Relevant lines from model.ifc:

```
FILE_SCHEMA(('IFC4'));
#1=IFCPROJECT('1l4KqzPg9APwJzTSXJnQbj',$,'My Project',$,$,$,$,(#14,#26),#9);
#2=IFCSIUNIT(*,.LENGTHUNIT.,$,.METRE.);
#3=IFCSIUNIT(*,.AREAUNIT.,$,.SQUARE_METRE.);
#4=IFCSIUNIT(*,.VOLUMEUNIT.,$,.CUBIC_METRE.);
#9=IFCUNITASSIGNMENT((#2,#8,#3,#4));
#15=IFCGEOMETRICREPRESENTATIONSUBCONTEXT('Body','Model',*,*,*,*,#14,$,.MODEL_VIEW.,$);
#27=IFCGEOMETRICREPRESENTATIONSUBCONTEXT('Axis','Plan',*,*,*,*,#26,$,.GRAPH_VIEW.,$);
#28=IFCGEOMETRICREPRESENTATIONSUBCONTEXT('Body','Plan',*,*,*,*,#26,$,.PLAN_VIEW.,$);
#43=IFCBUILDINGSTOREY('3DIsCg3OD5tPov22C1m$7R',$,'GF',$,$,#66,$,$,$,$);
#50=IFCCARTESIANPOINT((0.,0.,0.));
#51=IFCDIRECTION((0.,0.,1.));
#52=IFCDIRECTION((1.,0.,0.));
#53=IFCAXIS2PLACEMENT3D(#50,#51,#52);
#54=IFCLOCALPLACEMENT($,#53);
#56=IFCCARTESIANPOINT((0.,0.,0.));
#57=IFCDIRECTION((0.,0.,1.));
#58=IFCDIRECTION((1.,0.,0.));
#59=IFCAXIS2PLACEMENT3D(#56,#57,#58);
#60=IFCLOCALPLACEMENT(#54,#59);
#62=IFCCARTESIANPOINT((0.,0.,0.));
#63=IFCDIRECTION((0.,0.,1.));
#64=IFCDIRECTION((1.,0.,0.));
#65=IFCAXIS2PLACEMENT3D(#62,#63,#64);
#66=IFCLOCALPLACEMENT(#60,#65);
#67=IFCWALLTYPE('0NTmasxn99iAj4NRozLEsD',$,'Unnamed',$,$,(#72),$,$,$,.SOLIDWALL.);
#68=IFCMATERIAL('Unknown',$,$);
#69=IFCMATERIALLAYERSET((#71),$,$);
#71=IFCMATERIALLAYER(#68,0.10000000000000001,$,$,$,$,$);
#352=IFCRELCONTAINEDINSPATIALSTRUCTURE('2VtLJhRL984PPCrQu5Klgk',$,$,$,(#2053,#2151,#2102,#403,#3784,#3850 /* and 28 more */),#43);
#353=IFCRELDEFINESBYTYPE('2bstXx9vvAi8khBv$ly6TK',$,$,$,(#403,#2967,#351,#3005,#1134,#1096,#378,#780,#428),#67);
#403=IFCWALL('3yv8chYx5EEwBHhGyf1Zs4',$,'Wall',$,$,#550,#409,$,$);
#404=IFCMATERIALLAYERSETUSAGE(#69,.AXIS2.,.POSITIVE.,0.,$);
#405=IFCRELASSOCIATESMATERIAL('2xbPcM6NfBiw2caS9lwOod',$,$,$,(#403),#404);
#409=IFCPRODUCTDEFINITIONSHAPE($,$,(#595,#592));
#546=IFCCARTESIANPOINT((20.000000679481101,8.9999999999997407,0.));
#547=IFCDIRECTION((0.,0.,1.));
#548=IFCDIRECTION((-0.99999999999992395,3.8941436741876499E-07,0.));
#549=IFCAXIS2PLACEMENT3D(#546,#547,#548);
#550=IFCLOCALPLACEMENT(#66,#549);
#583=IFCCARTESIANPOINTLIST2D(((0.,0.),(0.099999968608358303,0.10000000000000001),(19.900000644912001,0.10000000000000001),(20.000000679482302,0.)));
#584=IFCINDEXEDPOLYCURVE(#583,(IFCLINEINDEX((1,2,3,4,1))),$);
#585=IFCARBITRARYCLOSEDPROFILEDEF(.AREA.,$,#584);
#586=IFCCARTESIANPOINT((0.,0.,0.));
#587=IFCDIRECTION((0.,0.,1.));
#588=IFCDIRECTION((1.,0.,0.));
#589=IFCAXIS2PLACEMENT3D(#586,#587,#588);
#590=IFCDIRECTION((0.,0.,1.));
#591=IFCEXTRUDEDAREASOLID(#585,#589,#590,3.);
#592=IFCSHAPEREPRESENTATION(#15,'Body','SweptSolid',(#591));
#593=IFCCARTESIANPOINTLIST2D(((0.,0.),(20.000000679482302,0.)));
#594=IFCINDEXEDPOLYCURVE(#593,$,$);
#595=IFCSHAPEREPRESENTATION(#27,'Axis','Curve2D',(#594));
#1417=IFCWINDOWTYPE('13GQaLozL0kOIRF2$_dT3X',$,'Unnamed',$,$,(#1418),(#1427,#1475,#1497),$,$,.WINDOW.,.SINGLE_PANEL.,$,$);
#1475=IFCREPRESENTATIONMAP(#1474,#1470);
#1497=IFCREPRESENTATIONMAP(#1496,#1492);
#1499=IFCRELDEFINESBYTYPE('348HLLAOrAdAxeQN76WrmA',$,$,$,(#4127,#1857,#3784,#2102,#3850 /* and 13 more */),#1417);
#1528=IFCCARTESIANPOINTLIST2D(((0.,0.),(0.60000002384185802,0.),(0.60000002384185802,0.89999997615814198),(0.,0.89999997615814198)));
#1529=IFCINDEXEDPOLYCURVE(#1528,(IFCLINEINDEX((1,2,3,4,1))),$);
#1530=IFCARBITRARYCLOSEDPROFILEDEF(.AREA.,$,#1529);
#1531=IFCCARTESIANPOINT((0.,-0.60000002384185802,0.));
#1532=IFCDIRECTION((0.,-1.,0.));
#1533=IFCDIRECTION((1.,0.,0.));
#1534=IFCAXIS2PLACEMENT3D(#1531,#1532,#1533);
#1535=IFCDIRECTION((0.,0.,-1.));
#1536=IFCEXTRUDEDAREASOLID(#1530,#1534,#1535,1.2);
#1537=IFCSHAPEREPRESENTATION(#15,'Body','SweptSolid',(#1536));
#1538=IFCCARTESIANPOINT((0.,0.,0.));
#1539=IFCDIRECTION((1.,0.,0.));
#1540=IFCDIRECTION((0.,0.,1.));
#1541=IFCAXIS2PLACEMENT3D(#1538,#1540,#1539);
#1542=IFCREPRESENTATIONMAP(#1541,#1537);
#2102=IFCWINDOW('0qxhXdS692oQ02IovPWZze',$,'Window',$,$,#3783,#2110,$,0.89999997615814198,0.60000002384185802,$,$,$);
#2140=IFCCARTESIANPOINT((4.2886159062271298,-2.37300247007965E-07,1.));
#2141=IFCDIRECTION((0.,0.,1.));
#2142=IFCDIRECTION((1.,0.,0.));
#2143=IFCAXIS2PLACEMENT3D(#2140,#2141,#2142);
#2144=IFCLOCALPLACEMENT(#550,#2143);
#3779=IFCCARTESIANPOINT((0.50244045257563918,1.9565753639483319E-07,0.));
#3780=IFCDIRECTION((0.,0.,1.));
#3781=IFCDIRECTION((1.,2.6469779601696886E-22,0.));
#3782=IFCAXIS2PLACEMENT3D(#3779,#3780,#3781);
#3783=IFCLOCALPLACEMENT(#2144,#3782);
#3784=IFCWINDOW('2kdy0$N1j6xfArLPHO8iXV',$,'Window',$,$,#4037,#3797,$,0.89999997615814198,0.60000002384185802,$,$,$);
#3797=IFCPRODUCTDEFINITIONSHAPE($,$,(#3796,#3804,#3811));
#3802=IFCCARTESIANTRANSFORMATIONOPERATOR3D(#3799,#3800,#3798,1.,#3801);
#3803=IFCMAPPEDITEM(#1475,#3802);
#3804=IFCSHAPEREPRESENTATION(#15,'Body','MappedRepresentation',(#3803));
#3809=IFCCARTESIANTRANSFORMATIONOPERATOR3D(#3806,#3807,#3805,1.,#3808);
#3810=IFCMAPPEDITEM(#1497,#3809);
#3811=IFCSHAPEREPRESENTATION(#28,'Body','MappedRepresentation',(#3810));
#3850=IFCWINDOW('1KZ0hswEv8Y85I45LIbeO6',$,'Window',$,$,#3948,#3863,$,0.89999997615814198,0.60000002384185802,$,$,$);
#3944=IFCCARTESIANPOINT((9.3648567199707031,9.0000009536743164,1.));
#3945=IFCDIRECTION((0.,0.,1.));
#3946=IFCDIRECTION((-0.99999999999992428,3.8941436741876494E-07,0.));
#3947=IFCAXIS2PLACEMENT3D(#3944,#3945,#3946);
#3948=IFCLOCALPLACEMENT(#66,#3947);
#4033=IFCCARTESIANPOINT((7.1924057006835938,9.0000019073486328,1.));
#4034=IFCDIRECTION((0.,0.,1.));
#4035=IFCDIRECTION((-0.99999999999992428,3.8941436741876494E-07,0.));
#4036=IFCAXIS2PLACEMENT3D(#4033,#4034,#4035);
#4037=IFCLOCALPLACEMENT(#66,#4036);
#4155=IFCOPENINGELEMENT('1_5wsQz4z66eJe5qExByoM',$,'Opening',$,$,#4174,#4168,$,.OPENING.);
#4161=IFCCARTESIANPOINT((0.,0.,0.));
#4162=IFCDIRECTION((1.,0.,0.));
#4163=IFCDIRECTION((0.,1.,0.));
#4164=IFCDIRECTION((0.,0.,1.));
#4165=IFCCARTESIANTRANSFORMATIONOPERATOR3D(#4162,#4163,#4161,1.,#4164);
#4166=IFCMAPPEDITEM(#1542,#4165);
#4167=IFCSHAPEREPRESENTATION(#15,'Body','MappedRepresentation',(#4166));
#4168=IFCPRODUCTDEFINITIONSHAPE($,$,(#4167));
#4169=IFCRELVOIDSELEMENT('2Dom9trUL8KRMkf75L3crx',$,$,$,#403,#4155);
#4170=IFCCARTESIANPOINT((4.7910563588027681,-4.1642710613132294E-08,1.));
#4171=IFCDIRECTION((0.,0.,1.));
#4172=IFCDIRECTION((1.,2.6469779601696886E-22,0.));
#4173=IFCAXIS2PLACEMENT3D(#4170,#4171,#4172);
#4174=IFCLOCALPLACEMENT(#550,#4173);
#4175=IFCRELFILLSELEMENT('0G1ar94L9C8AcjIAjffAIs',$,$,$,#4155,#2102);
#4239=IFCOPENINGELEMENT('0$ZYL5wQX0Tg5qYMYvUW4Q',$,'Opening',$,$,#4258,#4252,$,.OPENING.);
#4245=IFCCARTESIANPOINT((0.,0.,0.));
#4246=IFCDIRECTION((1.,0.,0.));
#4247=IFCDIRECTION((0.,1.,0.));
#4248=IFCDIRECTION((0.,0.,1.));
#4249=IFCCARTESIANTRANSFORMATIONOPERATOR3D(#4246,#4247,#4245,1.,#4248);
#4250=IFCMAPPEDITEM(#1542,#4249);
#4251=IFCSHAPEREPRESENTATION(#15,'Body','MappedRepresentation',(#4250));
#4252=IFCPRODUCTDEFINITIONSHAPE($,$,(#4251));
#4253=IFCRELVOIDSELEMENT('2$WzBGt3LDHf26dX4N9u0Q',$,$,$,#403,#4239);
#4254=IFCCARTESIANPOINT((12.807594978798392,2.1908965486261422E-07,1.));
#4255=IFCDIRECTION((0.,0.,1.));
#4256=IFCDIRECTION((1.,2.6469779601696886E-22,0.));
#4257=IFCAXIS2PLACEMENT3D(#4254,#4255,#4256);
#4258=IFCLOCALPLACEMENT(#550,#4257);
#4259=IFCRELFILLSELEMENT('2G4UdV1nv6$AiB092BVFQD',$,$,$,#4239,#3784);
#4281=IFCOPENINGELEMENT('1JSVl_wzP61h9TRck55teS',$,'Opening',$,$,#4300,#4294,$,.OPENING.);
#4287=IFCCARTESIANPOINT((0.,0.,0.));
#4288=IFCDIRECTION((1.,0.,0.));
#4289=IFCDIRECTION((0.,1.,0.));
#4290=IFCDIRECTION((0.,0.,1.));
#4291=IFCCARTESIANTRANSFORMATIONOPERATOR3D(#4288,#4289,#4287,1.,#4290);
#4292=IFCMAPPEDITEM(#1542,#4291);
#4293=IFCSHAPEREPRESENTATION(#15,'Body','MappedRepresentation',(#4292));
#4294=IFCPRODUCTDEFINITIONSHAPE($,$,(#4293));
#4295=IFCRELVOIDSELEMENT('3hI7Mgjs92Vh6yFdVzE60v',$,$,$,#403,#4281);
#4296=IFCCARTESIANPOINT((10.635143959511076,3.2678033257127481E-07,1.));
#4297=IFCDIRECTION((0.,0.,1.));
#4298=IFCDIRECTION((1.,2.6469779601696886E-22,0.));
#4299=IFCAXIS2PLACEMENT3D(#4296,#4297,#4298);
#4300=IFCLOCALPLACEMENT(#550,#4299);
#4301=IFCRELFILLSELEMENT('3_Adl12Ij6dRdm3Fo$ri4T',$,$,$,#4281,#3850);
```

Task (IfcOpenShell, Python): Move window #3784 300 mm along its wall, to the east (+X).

```python
import ifcopenshell
import ifcopenshell.api.geometry
import ifcopenshell.util.placement
import ifcopenshell.util.unit

model = ifcopenshell.open("model.ifc")
unit_scale = ifcopenshell.util.unit.calculate_unit_scale(model)

window = model.by_id(3784)
opening = window.FillsVoids[0].RelatingOpeningElement
wall = opening.VoidsElements[0].RelatingBuildingElement

wall_matrix = ifcopenshell.util.placement.get_local_placement(wall.ObjectPlacement)
shift = wall_matrix[:3, 0] * -0.3 / unit_scale
before = ifcopenshell.util.placement.get_local_placement(window.ObjectPlacement)[:3, 3].copy()

# The window is not placed relative to its opening, so move both.
for product in (opening, window):
    matrix = ifcopenshell.util.placement.get_local_placement(product.ObjectPlacement)
    matrix[:3, 3] += shift
    ifcopenshell.api.geometry.edit_object_placement(model, product=product, matrix=matrix, is_si=False)

after = ifcopenshell.util.placement.get_local_placement(window.ObjectPlacement)[:3, 3]
print("window moved by", (after - before).round(3) + 0.0)

model.write("model_rev.ifc")
```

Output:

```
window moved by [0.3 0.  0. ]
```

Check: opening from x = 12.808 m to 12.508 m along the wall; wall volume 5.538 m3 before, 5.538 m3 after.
